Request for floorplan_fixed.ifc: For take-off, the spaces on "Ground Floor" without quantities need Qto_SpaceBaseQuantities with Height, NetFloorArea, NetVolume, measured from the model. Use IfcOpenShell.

First a look at what the model holds.

```python
import ifcopenshell
import ifcopenshell.util.element
import ifcopenshell.util.unit

model = ifcopenshell.open("floorplan_fixed.ifc")
print(model.schema)
for unit_type in ("LENGTHUNIT", "AREAUNIT", "VOLUMEUNIT"):
    print(unit_type, ifcopenshell.util.unit.calculate_unit_scale(model, unit_type))
storey = next(s for s in model.by_type("IfcBuildingStorey") if s.Name == "Ground Floor")
spaces = [e for e in ifcopenshell.util.element.get_decomposition(storey) if e.is_a("IfcSpace")]
for e in sorted(spaces, key=lambda e: e.id()):
    print(e.id(), e.is_a(), e.Name, list(ifcopenshell.util.element.get_psets(e, qtos_only=True)), sep=" | ")
```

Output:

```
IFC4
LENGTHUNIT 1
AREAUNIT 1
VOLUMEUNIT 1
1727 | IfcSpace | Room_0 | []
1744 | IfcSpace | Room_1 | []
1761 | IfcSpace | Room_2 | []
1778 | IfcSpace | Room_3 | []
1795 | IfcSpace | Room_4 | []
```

```python
import ifcopenshell
import ifcopenshell.api.pset
import ifcopenshell.geom
import ifcopenshell.util.element
import ifcopenshell.util.shape
import ifcopenshell.util.unit

model = ifcopenshell.open("floorplan_fixed.ifc")
unit_scale = ifcopenshell.util.unit.calculate_unit_scale(model)
area_scale = ifcopenshell.util.unit.calculate_unit_scale(model, "AREAUNIT")
volume_scale = ifcopenshell.util.unit.calculate_unit_scale(model, "VOLUMEUNIT")
settings = ifcopenshell.geom.settings()

storey = next(s for s in model.by_type("IfcBuildingStorey") if s.Name == "Ground Floor")
spaces = [e for e in ifcopenshell.util.element.get_decomposition(storey) if e.is_a("IfcSpace")]

for e in sorted(spaces, key=lambda e: e.id()):
    if ifcopenshell.util.element.get_psets(e, qtos_only=True, should_inherit=False):
        continue
    # Geometry comes back in metres, in the element's own axes.
    shape = ifcopenshell.geom.create_shape(settings, e)
    values = {
        "Height": ifcopenshell.util.shape.get_z(shape.geometry) / unit_scale,
        "NetFloorArea": ifcopenshell.util.shape.get_footprint_area(shape.geometry) / area_scale,
        "NetVolume": ifcopenshell.util.shape.get_volume(shape.geometry) / volume_scale,
    }
    qto = ifcopenshell.api.pset.add_qto(model, product=e, name="Qto_SpaceBaseQuantities")
    ifcopenshell.api.pset.edit_qto(model, qto=qto, properties=values)
    print(e.id(), {k: round(v, 3) for k, v in values.items()})

model.write("floorplan_fixed_edited.ifc")
```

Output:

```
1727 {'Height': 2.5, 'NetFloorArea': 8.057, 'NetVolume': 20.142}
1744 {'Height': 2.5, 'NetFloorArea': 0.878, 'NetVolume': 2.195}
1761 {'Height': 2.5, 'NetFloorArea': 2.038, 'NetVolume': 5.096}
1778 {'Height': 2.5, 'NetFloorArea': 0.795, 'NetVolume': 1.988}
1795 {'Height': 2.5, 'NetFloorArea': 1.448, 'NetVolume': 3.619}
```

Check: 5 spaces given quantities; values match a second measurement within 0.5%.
